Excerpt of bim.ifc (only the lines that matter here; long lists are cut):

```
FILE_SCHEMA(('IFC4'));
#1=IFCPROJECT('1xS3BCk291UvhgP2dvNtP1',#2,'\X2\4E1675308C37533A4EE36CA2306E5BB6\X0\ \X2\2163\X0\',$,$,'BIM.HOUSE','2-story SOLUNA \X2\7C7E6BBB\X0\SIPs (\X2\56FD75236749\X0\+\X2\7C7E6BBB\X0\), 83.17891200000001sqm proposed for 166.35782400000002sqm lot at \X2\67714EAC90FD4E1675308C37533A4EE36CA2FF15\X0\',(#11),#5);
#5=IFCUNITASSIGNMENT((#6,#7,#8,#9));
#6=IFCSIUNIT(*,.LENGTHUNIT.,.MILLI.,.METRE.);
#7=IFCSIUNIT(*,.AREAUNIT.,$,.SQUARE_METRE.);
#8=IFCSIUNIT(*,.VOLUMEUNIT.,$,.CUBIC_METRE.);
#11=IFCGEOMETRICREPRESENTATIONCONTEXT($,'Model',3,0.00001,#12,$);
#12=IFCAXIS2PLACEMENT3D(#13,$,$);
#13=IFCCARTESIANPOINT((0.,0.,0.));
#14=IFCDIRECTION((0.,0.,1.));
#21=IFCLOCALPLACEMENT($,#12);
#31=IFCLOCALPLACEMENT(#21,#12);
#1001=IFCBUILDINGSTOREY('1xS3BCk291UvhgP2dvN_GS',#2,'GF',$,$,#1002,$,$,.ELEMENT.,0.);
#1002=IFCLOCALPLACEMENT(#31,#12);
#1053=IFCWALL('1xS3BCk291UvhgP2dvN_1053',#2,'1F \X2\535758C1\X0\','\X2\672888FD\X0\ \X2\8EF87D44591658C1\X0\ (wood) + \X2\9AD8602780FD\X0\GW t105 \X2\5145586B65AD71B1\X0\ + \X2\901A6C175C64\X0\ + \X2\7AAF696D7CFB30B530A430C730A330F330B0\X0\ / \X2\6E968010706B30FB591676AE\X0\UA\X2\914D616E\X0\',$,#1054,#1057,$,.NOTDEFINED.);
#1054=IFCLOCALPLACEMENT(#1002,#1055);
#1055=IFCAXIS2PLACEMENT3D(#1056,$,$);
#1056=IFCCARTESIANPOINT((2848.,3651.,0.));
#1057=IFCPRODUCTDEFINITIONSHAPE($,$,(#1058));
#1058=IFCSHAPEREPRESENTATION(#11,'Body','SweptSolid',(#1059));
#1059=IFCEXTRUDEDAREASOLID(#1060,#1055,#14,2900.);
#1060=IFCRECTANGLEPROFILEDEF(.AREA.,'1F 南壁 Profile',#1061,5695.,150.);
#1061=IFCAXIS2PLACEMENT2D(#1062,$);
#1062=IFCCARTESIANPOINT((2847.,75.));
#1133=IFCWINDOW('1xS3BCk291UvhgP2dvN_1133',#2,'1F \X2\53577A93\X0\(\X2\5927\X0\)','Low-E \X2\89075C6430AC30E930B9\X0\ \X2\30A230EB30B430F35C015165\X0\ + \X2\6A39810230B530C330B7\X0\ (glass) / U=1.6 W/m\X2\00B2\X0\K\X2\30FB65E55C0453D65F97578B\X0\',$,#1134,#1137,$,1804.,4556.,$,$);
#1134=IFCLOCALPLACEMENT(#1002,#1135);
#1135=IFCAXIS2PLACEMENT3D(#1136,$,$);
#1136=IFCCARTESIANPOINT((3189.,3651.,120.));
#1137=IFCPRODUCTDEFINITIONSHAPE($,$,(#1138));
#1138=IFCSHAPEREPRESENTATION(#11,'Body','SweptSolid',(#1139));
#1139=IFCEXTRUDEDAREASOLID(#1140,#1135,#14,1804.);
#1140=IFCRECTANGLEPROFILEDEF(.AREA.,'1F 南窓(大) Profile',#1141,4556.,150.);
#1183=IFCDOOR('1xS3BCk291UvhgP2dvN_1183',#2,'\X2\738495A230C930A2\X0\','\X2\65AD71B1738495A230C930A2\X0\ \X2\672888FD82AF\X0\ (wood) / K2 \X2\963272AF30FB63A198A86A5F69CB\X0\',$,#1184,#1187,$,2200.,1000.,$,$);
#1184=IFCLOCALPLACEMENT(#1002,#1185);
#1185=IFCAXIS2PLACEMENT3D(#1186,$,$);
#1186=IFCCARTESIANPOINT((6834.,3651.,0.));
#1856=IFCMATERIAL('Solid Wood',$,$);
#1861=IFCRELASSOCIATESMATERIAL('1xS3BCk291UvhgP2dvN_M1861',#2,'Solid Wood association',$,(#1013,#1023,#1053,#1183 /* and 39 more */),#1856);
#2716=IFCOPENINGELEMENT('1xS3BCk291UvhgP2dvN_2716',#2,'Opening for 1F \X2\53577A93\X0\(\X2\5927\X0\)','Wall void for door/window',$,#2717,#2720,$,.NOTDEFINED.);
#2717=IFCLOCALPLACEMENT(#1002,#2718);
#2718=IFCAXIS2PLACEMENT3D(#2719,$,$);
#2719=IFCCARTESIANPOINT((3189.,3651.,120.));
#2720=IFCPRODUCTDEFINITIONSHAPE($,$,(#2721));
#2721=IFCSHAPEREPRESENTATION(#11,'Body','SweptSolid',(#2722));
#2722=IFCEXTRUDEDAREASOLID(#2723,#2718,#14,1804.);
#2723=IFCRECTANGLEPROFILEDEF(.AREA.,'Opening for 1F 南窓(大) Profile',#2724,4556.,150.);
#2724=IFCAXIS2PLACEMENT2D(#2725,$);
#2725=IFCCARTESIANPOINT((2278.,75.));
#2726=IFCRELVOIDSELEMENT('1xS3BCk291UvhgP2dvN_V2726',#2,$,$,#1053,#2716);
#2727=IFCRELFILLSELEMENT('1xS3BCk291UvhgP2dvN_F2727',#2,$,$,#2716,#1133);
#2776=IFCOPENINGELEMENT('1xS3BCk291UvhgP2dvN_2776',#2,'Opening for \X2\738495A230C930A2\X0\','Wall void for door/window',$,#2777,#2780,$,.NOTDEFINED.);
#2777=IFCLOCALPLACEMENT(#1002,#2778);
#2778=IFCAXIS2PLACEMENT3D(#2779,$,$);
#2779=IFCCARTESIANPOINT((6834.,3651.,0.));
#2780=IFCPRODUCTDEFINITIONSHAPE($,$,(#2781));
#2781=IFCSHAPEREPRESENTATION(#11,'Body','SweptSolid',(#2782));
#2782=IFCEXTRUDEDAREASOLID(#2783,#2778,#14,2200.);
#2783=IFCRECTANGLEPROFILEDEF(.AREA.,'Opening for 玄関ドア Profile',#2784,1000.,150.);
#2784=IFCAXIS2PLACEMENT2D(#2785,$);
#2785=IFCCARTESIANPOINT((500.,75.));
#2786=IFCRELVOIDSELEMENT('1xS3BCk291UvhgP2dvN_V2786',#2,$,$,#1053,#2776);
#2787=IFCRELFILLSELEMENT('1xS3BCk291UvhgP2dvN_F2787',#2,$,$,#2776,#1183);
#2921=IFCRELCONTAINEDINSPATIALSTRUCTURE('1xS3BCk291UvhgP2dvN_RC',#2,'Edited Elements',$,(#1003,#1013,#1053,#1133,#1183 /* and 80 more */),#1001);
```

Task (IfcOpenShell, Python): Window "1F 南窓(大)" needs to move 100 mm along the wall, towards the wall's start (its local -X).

```python
import ifcopenshell
import ifcopenshell.api.geometry
import ifcopenshell.util.placement
import ifcopenshell.util.unit

model = ifcopenshell.open("bim.ifc")
unit_scale = ifcopenshell.util.unit.calculate_unit_scale(model)

window = model.by_id(1133)
opening = window.FillsVoids[0].RelatingOpeningElement
wall = opening.VoidsElements[0].RelatingBuildingElement

wall_matrix = ifcopenshell.util.placement.get_local_placement(wall.ObjectPlacement)
shift = wall_matrix[:3, 0] * -0.1 / unit_scale
before = ifcopenshell.util.placement.get_local_placement(window.ObjectPlacement)[:3, 3].copy()

# The window is not placed relative to its opening, so move both.
for product in (opening, window):
    matrix = ifcopenshell.util.placement.get_local_placement(product.ObjectPlacement)
    matrix[:3, 3] += shift
    ifcopenshell.api.geometry.edit_object_placement(model, product=product, matrix=matrix, is_si=False)

after = ifcopenshell.util.placement.get_local_placement(window.ObjectPlacement)[:3, 3]
print("window moved by", (after - before).round(3) + 0.0)

model.write("bim_v2.ifc")
```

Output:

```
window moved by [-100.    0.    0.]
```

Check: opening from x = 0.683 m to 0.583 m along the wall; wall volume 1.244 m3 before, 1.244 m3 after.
